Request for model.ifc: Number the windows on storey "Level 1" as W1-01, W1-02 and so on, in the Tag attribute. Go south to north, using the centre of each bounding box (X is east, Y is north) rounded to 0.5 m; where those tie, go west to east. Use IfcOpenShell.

First a look at what the model holds.

```python
import ifcopenshell
import ifcopenshell.util.element
import ifcopenshell.util.placement

model = ifcopenshell.open("model.ifc")
print(model.schema)
storey = next(s for s in model.by_type("IfcBuildingStorey") if s.Name == "Level 1")
windows = [e for e in ifcopenshell.util.element.get_decomposition(storey) if e.is_a("IfcWindow")]
for e in sorted(windows, key=lambda e: e.id()):
    origin = ifcopenshell.util.placement.get_local_placement(e.ObjectPlacement)[:3, 3]
    print(e.id(), e.Tag, e.Name, origin.round(2) + 0.0, sep=" | ")
```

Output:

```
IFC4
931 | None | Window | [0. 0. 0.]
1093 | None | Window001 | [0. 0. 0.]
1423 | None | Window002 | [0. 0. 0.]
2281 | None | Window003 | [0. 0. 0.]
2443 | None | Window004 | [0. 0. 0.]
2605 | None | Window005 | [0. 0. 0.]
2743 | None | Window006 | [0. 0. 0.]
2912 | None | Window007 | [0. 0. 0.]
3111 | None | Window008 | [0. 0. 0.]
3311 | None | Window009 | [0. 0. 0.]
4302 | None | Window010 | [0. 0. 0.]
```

```python
import ifcopenshell
import ifcopenshell.geom
import ifcopenshell.util.element
import ifcopenshell.util.shape

model = ifcopenshell.open("model.ifc")
settings = ifcopenshell.geom.settings()
settings.set("use-world-coords", True)


def centre(element):
    shape = ifcopenshell.geom.create_shape(settings, element)
    return ifcopenshell.util.shape.get_bbox_centroid(shape.geometry)


storey = next(s for s in model.by_type("IfcBuildingStorey") if s.Name == "Level 1")
windows = [e for e in ifcopenshell.util.element.get_decomposition(storey) if e.is_a("IfcWindow")]

# Insertion points can sit at a corner or the storey origin, so sort by the geometry (in metres).
centres = {e: centre(e) for e in windows}
windows.sort(key=lambda e: (round(centres[e][1] / 0.5), centres[e][0]))

for i, e in enumerate(windows, start=1):
    number = f"W1-{i:02d}"
    e.Tag = number
    print(e.id(), number)

model.write("model_updated.ifc")
```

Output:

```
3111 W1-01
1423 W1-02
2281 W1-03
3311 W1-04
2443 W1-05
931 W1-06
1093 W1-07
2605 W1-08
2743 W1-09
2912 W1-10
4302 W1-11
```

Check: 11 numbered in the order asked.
